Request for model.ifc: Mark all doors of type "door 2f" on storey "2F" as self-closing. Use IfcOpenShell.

First a look at what the model holds.

```python
import ifcopenshell
import ifcopenshell.util.element

model = ifcopenshell.open("model.ifc")
print(model.schema)
storey = next(s for s in model.by_type("IfcBuildingStorey") if s.Name == "2F")
doors = [e for e in ifcopenshell.util.element.get_decomposition(storey) if e.is_a("IfcDoor")]
seen = {}
for e in doors:
    element_type = ifcopenshell.util.element.get_type(e)
    key = (element_type.Name if element_type != e and element_type else None, ifcopenshell.util.element.get_pset(e, "Pset_DoorCommon", "SelfClosing"))
    seen[key] = seen.get(key, 0) + 1
for (name, value), count in sorted(seen.items(), key=str):
    print(count, "x", name, "|", value)
```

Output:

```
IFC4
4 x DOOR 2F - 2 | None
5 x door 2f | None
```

```python
import ifcopenshell
import ifcopenshell.api.pset
import ifcopenshell.util.element

model = ifcopenshell.open("model.ifc")

storey = next(s for s in model.by_type("IfcBuildingStorey") if s.Name == "2F")
doors = [e for e in ifcopenshell.util.element.get_decomposition(storey) if e.is_a("IfcDoor")]

count = 0
for e in doors:
    element_type = ifcopenshell.util.element.get_type(e)
    if element_type in (None, e) or element_type.Name != "door 2f":
        continue
    # add_pset returns the element's existing set when there is one.
    pset = ifcopenshell.api.pset.add_pset(model, product=e, name="Pset_DoorCommon")
    ifcopenshell.api.pset.edit_pset(model, pset=pset, properties={"SelfClosing": True})
    count += 1

print(count, "doors updated")

model.write("model_rev.ifc")
```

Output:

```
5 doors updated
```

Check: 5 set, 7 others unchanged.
